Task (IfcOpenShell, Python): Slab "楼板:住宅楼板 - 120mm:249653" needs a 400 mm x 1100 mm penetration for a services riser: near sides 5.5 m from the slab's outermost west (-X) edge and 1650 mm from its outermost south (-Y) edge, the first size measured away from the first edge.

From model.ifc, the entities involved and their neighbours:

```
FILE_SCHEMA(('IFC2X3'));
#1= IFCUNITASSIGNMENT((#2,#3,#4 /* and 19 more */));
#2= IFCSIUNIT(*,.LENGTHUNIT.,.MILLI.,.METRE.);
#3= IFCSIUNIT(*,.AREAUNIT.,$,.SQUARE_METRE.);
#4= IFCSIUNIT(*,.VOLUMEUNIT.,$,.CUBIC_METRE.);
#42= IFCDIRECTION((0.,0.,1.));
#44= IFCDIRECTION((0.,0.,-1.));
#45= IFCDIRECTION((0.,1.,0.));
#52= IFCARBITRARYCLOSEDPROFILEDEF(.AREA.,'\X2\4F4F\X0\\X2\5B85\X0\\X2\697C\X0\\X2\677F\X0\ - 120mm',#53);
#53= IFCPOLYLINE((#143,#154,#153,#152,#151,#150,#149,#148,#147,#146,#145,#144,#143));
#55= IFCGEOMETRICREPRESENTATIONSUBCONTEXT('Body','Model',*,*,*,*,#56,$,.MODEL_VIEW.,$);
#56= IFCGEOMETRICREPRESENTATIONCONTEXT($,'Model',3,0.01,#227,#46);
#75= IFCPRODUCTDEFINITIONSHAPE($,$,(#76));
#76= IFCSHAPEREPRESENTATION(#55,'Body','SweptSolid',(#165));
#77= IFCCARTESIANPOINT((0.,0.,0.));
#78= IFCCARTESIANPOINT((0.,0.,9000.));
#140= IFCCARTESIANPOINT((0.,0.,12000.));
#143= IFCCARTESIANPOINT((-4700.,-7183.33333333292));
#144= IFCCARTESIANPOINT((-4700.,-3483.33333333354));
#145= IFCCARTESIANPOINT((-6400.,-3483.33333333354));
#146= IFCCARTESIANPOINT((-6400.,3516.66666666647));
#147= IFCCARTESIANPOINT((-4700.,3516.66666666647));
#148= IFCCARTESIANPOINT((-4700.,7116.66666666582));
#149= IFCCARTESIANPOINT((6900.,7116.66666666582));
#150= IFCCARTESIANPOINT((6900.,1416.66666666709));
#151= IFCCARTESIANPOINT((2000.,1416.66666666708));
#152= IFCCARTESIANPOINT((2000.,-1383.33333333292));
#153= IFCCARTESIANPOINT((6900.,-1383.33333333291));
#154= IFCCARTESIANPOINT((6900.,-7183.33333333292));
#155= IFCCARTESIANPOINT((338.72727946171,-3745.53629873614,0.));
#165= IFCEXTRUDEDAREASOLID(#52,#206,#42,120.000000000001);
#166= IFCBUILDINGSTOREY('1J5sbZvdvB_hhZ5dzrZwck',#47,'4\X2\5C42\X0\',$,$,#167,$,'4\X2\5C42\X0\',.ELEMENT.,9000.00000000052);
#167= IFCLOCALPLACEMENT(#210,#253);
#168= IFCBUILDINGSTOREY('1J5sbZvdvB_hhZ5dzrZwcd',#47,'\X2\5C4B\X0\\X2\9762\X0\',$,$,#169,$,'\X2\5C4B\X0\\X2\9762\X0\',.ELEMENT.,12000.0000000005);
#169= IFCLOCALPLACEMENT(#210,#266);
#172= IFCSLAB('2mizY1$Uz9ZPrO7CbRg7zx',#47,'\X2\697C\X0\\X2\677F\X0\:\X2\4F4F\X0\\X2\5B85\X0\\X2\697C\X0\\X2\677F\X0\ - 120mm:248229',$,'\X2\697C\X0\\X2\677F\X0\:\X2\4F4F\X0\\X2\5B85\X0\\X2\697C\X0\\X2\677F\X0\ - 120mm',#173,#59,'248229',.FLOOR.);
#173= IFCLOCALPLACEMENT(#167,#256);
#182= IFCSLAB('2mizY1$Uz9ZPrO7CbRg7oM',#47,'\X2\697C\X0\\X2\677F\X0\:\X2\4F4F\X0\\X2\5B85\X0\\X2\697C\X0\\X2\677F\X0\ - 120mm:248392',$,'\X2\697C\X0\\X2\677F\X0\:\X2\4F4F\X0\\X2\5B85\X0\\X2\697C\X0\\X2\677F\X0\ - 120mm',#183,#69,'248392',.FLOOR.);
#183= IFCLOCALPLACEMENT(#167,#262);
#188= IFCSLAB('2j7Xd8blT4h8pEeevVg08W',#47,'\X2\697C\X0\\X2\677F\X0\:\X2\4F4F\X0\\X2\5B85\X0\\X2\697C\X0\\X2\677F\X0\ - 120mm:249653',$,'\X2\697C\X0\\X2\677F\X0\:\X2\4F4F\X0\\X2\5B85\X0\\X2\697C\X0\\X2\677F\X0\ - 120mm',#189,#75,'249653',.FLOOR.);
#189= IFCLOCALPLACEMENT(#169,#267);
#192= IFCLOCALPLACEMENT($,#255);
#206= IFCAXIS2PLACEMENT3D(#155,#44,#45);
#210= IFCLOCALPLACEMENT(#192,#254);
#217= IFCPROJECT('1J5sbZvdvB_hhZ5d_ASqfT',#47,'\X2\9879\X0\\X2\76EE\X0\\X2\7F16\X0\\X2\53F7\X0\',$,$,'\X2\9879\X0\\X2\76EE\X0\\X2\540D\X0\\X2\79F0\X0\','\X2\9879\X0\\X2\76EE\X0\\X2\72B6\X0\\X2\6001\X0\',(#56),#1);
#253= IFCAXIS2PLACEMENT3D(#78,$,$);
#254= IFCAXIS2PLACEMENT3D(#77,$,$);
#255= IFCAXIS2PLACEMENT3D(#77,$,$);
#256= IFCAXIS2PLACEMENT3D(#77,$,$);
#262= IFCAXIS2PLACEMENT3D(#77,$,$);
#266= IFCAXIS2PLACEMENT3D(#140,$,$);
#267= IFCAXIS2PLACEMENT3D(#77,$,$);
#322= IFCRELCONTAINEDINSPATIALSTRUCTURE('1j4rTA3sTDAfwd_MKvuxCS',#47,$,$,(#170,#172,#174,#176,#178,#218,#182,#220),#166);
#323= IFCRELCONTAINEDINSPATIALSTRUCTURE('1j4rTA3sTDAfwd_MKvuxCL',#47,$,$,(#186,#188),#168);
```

```python
import numpy as np
import ifcopenshell
import ifcopenshell.api.feature
import ifcopenshell.api.geometry
import ifcopenshell.api.root
import ifcopenshell.geom
import ifcopenshell.util.placement
import ifcopenshell.util.representation
import ifcopenshell.util.shape
import ifcopenshell.util.unit

model = ifcopenshell.open("model.ifc")
unit_scale = ifcopenshell.util.unit.calculate_unit_scale(model)
settings = ifcopenshell.geom.settings()


def volume(element):
    """Net volume in cubic metres, openings subtracted."""
    shape = ifcopenshell.geom.create_shape(settings, element)
    return ifcopenshell.util.shape.get_volume(shape.geometry)


slab = model.by_guid("2j7Xd8blT4h8pEeevVg08W")
before = volume(slab)

# Extent in the slab's own axes, in metres. The edges named are its -X and -Y sides.
slab_shape = ifcopenshell.geom.create_shape(settings, slab)
vertices = ifcopenshell.util.shape.get_vertices(slab_shape.geometry)
x_min, y_min, bottom = vertices.min(axis=0)
top = vertices[:, 2].max()

opening = ifcopenshell.api.root.create_entity(model, ifc_class="IfcOpeningElement", name="Services riser opening")
context = ifcopenshell.util.representation.get_context(model, "Model", "Body", "MODEL_VIEW")
width, depth = 0.4, 1.1
outline = [(0.0, 0.0), (width, 0.0), (width, depth), (0.0, depth), (0.0, 0.0)]
# Overshoot both faces by 50 mm so the cut is clean.
shape = ifcopenshell.api.geometry.add_slab_representation(
    model, context=context, depth=top - bottom + 0.1, polyline=outline
)
ifcopenshell.api.geometry.assign_representation(model, product=opening, representation=shape)

matrix = ifcopenshell.util.placement.get_local_placement(slab.ObjectPlacement)
matrix[:, 3] = matrix @ np.append(np.array([x_min + 5.5, y_min + 1.65, bottom - 0.05]) / unit_scale, 1.0)
ifcopenshell.api.geometry.edit_object_placement(model, product=opening, matrix=matrix, is_si=False)
ifcopenshell.api.feature.add_feature(model, feature=opening, element=slab)

after = volume(slab)

print(f"slab volume {before:.3f} -> {after:.3f} m3")

model.write("model-out.ifc")
```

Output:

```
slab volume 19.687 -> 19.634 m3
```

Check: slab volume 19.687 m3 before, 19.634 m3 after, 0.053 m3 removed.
